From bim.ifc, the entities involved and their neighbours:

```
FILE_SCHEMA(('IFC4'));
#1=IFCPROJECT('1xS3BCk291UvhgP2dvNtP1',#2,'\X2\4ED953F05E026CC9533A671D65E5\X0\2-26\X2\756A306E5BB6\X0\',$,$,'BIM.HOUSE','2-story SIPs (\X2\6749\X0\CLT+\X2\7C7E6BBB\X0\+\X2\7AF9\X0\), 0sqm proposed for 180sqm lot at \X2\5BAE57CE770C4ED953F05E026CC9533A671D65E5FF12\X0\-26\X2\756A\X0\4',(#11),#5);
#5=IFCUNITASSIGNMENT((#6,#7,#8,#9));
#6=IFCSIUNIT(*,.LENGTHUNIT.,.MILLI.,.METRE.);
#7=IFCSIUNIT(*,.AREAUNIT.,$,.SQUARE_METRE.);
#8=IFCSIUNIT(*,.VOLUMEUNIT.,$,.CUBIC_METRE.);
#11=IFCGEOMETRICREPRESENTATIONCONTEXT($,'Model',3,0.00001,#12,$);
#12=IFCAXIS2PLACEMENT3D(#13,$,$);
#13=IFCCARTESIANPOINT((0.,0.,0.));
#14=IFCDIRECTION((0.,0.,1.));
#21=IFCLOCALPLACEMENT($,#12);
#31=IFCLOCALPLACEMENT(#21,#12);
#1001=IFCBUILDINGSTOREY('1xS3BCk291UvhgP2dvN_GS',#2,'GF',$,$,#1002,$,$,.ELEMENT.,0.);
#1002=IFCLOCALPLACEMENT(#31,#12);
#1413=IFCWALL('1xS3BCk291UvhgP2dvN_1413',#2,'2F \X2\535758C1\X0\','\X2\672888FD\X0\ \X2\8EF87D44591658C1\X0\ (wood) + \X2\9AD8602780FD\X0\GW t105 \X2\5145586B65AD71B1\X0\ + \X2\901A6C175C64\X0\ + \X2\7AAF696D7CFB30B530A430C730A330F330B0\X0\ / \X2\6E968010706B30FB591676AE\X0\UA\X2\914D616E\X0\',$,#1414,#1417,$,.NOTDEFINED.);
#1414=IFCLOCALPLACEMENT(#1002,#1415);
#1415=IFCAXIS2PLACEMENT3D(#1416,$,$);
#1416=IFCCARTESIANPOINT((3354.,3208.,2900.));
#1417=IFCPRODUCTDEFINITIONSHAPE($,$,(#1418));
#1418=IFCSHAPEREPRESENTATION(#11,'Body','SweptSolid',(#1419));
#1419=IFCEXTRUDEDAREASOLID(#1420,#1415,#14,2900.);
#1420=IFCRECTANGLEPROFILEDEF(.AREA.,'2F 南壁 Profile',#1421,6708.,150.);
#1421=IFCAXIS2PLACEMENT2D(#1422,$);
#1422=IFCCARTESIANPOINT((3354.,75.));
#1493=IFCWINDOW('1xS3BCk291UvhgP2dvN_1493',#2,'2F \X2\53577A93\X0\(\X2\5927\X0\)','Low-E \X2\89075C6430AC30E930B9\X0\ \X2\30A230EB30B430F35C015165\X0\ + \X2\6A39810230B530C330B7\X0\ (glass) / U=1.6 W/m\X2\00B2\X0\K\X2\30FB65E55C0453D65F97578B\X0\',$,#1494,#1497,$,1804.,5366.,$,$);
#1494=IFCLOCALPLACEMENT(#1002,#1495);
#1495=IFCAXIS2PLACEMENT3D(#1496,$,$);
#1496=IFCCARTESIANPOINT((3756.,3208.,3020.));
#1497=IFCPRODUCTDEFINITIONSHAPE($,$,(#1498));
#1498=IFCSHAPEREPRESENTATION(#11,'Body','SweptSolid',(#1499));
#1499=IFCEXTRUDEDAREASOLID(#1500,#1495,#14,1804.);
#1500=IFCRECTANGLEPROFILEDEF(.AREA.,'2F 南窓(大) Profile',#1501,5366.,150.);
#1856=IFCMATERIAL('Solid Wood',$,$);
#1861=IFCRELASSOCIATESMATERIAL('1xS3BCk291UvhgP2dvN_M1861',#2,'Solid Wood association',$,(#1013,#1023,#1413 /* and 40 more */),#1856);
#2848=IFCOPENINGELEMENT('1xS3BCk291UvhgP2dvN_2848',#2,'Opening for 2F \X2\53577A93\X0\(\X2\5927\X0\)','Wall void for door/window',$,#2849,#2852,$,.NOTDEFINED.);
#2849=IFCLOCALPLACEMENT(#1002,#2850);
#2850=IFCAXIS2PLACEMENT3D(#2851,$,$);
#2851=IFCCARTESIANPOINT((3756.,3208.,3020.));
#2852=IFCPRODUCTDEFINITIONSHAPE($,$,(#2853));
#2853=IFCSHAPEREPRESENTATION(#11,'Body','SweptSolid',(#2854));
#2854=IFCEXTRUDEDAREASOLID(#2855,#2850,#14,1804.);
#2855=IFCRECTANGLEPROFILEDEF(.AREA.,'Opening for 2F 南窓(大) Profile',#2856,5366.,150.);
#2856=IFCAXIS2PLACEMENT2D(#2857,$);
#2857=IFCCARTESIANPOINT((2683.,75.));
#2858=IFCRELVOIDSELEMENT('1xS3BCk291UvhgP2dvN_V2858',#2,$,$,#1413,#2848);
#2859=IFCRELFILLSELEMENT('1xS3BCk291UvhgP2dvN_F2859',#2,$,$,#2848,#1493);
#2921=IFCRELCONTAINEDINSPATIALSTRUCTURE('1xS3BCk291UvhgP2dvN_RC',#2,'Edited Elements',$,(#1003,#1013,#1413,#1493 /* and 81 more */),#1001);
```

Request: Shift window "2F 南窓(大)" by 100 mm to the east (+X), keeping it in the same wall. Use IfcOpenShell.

```python
import ifcopenshell
import ifcopenshell.api.geometry
import ifcopenshell.util.placement
import ifcopenshell.util.unit

model = ifcopenshell.open("bim.ifc")
unit_scale = ifcopenshell.util.unit.calculate_unit_scale(model)

window = model.by_id(1493)
opening = window.FillsVoids[0].RelatingOpeningElement
wall = opening.VoidsElements[0].RelatingBuildingElement

wall_matrix = ifcopenshell.util.placement.get_local_placement(wall.ObjectPlacement)
shift = wall_matrix[:3, 0] * 0.1 / unit_scale
before = ifcopenshell.util.placement.get_local_placement(window.ObjectPlacement)[:3, 3].copy()

# The window is not placed relative to its opening, so move both.
for product in (opening, window):
    matrix = ifcopenshell.util.placement.get_local_placement(product.ObjectPlacement)
    matrix[:3, 3] += shift
    ifcopenshell.api.geometry.edit_object_placement(model, product=product, matrix=matrix, is_si=False)

after = ifcopenshell.util.placement.get_local_placement(window.ObjectPlacement)[:3, 3]
print("window moved by", (after - before).round(3) + 0.0)

model.write("bim_rev.ifc")
```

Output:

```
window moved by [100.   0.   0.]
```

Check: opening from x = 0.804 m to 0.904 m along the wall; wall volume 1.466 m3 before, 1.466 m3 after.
